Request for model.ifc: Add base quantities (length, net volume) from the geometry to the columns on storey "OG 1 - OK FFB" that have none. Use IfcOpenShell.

First a look at what the model holds.

```python
import ifcopenshell
import ifcopenshell.util.element
import ifcopenshell.util.unit

model = ifcopenshell.open("model.ifc")
print(model.schema)
for unit_type in ("LENGTHUNIT", "AREAUNIT", "VOLUMEUNIT"):
    print(unit_type, ifcopenshell.util.unit.calculate_unit_scale(model, unit_type))
storey = next(s for s in model.by_type("IfcBuildingStorey") if s.Name == "OG 1 - OK FFB")
columns = [e for e in ifcopenshell.util.element.get_decomposition(storey) if e.is_a("IfcColumn")]
for e in sorted(columns, key=lambda e: e.id()):
    print(e.id(), e.is_a(), e.Name, list(ifcopenshell.util.element.get_psets(e, qtos_only=True)), sep=" | ")
```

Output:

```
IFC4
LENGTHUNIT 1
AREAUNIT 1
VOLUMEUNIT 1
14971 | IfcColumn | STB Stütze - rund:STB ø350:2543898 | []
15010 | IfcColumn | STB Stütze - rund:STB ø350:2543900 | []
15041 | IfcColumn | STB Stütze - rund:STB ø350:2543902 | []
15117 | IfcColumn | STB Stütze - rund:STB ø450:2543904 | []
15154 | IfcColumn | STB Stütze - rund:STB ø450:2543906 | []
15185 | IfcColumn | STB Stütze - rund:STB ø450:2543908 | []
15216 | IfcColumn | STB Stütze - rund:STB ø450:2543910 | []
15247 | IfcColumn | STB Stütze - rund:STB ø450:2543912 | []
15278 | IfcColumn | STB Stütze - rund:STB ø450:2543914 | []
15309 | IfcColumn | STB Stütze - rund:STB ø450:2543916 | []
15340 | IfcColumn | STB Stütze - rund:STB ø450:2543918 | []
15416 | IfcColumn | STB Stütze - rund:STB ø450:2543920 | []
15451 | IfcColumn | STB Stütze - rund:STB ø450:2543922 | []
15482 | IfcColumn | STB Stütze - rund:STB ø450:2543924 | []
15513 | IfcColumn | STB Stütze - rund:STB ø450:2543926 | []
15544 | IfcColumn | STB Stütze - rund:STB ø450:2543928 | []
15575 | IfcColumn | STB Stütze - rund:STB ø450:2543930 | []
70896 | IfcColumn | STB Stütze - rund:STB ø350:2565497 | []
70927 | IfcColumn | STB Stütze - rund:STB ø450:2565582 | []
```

```python
import ifcopenshell
import ifcopenshell.api.pset
import ifcopenshell.geom
import ifcopenshell.util.element
import ifcopenshell.util.shape
import ifcopenshell.util.unit

model = ifcopenshell.open("model.ifc")
unit_scale = ifcopenshell.util.unit.calculate_unit_scale(model)
volume_scale = ifcopenshell.util.unit.calculate_unit_scale(model, "VOLUMEUNIT")
settings = ifcopenshell.geom.settings()

storey = next(s for s in model.by_type("IfcBuildingStorey") if s.Name == "OG 1 - OK FFB")
columns = [e for e in ifcopenshell.util.element.get_decomposition(storey) if e.is_a("IfcColumn")]

for e in sorted(columns, key=lambda e: e.id()):
    if ifcopenshell.util.element.get_psets(e, qtos_only=True, should_inherit=False):
        continue
    # Geometry comes back in metres, in the element's own axes.
    shape = ifcopenshell.geom.create_shape(settings, e)
    values = {
        "Length": ifcopenshell.util.shape.get_z(shape.geometry) / unit_scale,
        "NetVolume": ifcopenshell.util.shape.get_volume(shape.geometry) / volume_scale,
    }
    qto = ifcopenshell.api.pset.add_qto(model, product=e, name="Qto_ColumnBaseQuantities")
    ifcopenshell.api.pset.edit_qto(model, qto=qto, properties=values)
    print(e.id(), {k: round(v, 3) for k, v in values.items()})

model.write("model_rev.ifc")
```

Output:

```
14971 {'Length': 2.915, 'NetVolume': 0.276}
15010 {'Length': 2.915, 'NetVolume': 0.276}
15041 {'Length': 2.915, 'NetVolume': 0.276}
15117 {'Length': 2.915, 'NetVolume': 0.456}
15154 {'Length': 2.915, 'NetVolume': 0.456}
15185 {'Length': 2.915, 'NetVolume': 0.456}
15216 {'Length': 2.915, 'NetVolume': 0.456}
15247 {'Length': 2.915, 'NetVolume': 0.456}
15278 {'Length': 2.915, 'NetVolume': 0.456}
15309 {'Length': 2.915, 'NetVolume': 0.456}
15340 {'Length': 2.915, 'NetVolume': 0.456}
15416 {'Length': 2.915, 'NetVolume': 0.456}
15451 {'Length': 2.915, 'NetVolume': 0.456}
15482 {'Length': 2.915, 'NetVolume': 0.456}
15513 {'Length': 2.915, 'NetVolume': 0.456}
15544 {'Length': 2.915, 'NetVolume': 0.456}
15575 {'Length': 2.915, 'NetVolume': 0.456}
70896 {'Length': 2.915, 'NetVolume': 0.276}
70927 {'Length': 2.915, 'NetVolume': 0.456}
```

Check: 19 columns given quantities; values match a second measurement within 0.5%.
